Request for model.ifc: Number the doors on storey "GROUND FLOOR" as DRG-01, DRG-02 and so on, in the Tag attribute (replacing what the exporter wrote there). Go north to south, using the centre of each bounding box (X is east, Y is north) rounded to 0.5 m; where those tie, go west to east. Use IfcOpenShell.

First a look at what the model holds.

```python
import ifcopenshell
import ifcopenshell.util.element
import ifcopenshell.util.placement

model = ifcopenshell.open("model.ifc")
print(model.schema)
storey = next(s for s in model.by_type("IfcBuildingStorey") if s.Name == "GROUND FLOOR")
doors = [e for e in ifcopenshell.util.element.get_decomposition(storey) if e.is_a("IfcDoor")]
for e in sorted(doors, key=lambda e: e.id()):
    origin = ifcopenshell.util.placement.get_local_placement(e.ObjectPlacement)[:3, 3]
    print(e.id(), e.Tag, e.Name, origin.round(2) + 0.0, sep=" | ")
```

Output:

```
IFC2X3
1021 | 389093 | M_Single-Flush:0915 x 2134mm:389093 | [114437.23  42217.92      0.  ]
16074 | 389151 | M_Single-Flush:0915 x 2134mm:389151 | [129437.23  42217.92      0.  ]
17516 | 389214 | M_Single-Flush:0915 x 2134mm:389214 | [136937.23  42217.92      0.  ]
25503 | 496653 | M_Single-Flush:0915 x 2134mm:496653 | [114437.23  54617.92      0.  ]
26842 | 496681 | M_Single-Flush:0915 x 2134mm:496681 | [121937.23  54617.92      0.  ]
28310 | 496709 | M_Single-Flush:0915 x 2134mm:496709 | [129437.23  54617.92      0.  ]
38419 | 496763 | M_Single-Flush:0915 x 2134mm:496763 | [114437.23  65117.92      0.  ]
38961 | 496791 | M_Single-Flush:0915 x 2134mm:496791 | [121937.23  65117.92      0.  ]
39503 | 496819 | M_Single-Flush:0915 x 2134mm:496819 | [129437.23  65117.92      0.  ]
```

```python
import ifcopenshell
import ifcopenshell.geom
import ifcopenshell.util.element
import ifcopenshell.util.shape

model = ifcopenshell.open("model.ifc")
settings = ifcopenshell.geom.settings()
settings.set("use-world-coords", True)


def centre(element):
    shape = ifcopenshell.geom.create_shape(settings, element)
    return ifcopenshell.util.shape.get_bbox_centroid(shape.geometry)


storey = next(s for s in model.by_type("IfcBuildingStorey") if s.Name == "GROUND FLOOR")
doors = [e for e in ifcopenshell.util.element.get_decomposition(storey) if e.is_a("IfcDoor")]

# Insertion points can sit at a corner or the storey origin, so sort by the geometry (in metres).
centres = {e: centre(e) for e in doors}
doors.sort(key=lambda e: (-round(centres[e][1] / 0.5), centres[e][0]))

for i, e in enumerate(doors, start=1):
    number = f"DRG-{i:02d}"
    e.Tag = number
    print(e.id(), number)

model.write("model_edited.ifc")
```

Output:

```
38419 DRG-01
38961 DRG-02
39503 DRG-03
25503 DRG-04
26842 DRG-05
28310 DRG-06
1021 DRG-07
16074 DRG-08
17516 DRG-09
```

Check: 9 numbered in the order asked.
